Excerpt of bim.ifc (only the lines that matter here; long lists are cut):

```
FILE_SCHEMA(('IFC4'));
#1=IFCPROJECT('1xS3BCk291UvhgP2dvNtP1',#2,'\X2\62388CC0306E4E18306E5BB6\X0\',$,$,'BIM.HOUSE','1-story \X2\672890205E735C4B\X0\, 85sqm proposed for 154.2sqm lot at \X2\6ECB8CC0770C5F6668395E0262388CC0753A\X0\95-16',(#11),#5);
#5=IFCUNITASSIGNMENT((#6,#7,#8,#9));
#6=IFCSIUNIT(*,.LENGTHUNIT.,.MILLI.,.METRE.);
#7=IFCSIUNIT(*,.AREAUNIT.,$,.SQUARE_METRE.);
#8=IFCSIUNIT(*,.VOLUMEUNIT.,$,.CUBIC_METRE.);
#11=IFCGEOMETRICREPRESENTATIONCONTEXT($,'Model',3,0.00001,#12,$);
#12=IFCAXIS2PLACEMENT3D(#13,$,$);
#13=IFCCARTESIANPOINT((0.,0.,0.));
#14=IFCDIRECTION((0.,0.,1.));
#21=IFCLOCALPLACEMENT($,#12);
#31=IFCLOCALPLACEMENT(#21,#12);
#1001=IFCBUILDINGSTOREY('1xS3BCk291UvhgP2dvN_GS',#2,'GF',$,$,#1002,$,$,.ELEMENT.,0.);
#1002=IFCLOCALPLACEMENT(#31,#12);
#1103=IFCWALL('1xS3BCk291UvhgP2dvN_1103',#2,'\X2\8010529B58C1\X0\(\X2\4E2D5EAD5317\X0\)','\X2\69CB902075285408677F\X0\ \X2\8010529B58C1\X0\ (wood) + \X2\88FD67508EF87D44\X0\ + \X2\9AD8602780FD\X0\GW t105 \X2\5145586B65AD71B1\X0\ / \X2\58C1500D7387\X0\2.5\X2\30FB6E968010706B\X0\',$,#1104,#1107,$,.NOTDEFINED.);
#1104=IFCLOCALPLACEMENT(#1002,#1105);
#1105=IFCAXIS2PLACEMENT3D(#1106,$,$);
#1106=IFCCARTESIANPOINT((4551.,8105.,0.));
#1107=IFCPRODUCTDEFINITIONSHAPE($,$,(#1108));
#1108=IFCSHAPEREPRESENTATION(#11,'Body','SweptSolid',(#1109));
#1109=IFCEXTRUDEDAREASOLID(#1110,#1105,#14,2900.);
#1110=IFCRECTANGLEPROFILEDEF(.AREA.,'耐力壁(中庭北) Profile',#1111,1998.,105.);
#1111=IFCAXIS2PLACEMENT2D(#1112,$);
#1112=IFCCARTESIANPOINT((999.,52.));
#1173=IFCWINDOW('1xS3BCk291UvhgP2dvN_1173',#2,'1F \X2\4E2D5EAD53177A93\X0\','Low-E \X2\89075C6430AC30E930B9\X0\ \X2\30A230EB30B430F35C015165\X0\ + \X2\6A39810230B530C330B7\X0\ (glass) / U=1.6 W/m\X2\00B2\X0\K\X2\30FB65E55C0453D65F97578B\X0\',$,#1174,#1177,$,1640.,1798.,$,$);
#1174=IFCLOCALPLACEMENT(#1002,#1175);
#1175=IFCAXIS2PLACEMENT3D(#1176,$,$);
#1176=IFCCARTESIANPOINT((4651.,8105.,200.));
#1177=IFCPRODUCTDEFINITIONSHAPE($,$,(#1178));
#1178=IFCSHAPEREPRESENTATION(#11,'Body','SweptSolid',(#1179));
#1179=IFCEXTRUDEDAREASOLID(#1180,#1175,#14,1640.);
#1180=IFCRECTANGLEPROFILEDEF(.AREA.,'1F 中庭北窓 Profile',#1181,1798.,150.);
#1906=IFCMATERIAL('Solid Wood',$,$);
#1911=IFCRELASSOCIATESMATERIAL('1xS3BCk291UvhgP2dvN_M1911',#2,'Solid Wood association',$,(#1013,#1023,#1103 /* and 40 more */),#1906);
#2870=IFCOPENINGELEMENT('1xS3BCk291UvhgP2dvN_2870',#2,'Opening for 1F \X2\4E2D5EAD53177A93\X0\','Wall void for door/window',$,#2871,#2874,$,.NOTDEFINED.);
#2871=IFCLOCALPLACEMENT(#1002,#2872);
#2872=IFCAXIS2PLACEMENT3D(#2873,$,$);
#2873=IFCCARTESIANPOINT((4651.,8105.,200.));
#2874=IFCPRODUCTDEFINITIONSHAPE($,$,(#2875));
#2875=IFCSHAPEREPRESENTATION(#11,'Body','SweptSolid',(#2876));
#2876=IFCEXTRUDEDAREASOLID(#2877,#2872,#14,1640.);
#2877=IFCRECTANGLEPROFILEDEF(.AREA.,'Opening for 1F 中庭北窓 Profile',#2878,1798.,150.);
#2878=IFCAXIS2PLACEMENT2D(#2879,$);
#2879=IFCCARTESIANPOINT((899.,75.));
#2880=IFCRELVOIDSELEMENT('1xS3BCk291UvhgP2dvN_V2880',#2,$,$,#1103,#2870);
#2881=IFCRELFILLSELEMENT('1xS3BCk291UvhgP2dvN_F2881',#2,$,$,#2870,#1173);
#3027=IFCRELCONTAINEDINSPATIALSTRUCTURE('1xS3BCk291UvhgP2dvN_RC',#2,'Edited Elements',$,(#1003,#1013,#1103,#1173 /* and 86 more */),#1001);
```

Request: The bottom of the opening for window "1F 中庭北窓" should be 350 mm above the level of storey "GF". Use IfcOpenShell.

```python
import numpy as np
import ifcopenshell
import ifcopenshell.api.geometry
import ifcopenshell.geom
import ifcopenshell.util.element
import ifcopenshell.util.placement
import ifcopenshell.util.shape
import ifcopenshell.util.unit

model = ifcopenshell.open("bim.ifc")
unit_scale = ifcopenshell.util.unit.calculate_unit_scale(model)

window = model.by_guid("1xS3BCk291UvhgP2dvN_1173")
opening = window.FillsVoids[0].RelatingOpeningElement
storey = ifcopenshell.util.element.get_container(window, ifc_class="IfcBuildingStorey")
level = ifcopenshell.util.placement.get_local_placement(storey.ObjectPlacement)[2, 3]

# The opening's origin need not be at the sill, so measure its lowest point.
shape = ifcopenshell.geom.create_shape(ifcopenshell.geom.settings(), opening)
bottom = ifcopenshell.util.shape.get_shape_bottom_elevation(shape, shape.geometry) / unit_scale
dz = level + 350.0 - bottom

shift = np.array([0.0, 0.0, dz])
# The window is not placed relative to its opening, so move both.
for product in (opening, window):
    matrix = ifcopenshell.util.placement.get_local_placement(product.ObjectPlacement)
    matrix[:3, 3] += shift
    ifcopenshell.api.geometry.edit_object_placement(model, product=product, matrix=matrix, is_si=False)

print(f"moved by {dz * unit_scale:+.3f} m")

model.write("bim-out.ifc")
```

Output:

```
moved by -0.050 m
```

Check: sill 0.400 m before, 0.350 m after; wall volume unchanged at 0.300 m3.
